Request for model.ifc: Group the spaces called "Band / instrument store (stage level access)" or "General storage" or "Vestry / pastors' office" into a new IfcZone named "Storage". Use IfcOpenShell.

First a look at what the model holds.

```python
import ifcopenshell

model = ifcopenshell.open("model.ifc")
print(model.schema)
seen = {}
for space in model.by_type("IfcSpace"):
    seen[space.LongName] = seen.get(space.LongName, 0) + 1
for name, count in sorted(seen.items(), key=str):
    print(count, "x", name)
print("zones:", [z.Name for z in model.by_type("IfcZone")][:20])
```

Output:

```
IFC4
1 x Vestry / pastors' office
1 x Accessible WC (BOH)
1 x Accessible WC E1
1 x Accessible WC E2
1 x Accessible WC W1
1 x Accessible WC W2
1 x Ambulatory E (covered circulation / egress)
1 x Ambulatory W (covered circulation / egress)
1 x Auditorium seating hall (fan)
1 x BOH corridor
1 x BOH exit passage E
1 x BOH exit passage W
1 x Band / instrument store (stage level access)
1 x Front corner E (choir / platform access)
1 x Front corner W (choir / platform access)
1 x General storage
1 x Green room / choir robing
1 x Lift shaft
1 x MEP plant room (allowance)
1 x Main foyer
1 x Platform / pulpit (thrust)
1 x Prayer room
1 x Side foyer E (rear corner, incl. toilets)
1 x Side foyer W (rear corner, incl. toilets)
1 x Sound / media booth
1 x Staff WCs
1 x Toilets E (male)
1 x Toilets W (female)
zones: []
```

```python
import ifcopenshell
import ifcopenshell.api.group
import ifcopenshell.api.root

model = ifcopenshell.open("model.ifc")

names = {"Band / instrument store (stage level access)", "General storage", "Vestry / pastors' office"}
spaces = [s for s in model.by_type("IfcSpace") if s.LongName in names]

zone = ifcopenshell.api.root.create_entity(model, ifc_class="IfcZone", name="Storage")
ifcopenshell.api.group.assign_group(model, products=spaces, group=zone)
print(len(spaces), "spaces in", zone.Name)

model.write("model_edited.ifc")
```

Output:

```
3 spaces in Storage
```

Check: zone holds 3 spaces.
